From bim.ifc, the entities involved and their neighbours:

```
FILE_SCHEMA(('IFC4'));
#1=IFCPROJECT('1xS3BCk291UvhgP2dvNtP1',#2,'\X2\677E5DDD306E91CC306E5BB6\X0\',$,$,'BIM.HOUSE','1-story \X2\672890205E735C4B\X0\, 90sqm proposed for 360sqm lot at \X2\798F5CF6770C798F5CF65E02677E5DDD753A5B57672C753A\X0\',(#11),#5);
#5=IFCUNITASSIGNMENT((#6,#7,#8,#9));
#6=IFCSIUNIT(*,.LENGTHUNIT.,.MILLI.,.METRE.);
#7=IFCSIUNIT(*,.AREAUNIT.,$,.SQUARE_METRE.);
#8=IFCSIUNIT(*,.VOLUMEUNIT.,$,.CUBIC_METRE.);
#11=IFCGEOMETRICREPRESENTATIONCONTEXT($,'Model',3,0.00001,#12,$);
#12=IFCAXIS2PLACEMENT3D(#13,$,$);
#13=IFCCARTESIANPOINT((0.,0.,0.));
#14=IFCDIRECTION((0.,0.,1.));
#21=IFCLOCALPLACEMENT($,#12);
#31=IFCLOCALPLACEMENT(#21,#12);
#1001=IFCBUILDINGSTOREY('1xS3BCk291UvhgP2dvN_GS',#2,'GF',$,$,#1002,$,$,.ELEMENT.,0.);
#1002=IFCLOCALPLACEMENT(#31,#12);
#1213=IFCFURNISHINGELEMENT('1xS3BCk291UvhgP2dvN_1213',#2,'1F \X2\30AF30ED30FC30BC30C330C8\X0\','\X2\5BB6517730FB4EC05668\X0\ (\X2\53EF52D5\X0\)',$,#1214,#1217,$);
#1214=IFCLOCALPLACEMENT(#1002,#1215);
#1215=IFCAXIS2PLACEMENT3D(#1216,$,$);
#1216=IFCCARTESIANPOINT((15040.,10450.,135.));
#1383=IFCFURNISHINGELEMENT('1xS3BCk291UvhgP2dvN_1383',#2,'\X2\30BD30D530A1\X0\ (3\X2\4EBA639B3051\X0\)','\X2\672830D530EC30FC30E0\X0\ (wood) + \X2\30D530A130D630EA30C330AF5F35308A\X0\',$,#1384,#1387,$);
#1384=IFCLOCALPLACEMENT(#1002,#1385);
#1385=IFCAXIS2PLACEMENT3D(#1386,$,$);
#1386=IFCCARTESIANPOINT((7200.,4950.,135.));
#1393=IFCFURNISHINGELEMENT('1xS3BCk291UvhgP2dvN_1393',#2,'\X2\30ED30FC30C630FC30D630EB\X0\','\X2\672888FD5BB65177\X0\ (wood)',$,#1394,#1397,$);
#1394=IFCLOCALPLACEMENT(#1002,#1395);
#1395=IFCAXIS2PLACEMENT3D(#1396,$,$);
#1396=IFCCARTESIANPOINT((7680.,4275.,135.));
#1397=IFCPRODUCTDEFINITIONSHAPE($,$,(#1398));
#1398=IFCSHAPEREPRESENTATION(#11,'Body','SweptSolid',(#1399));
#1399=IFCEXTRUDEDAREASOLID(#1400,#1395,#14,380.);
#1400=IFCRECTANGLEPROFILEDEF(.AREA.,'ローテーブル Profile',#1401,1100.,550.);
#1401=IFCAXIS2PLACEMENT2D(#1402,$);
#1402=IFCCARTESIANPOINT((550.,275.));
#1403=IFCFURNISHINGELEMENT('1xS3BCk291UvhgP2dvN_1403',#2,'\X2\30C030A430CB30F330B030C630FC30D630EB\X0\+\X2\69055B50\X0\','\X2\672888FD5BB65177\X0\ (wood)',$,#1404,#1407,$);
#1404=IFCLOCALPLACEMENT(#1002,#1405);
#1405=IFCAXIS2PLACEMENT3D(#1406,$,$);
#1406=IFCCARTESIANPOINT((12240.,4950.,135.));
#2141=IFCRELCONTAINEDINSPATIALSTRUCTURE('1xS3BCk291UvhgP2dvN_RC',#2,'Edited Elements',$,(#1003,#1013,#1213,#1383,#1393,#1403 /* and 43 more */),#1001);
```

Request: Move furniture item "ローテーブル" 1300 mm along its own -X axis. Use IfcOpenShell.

```python
import ifcopenshell
import ifcopenshell.api.geometry
import ifcopenshell.util.placement

model = ifcopenshell.open("bim.ifc")

item = model.by_id(1393)
matrix = ifcopenshell.util.placement.get_local_placement(item.ObjectPlacement)
matrix[:3, 3] -= matrix[:3, 0] * 1300.0
ifcopenshell.api.geometry.edit_object_placement(model, product=item, matrix=matrix, is_si=False)

print(ifcopenshell.util.placement.get_local_placement(item.ObjectPlacement).round(3) + 0.0)

model.write("bim_edited.ifc")
```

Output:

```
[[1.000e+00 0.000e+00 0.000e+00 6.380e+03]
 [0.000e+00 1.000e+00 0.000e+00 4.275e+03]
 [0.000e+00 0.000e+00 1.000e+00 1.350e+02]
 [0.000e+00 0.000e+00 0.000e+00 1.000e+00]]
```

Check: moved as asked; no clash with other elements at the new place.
